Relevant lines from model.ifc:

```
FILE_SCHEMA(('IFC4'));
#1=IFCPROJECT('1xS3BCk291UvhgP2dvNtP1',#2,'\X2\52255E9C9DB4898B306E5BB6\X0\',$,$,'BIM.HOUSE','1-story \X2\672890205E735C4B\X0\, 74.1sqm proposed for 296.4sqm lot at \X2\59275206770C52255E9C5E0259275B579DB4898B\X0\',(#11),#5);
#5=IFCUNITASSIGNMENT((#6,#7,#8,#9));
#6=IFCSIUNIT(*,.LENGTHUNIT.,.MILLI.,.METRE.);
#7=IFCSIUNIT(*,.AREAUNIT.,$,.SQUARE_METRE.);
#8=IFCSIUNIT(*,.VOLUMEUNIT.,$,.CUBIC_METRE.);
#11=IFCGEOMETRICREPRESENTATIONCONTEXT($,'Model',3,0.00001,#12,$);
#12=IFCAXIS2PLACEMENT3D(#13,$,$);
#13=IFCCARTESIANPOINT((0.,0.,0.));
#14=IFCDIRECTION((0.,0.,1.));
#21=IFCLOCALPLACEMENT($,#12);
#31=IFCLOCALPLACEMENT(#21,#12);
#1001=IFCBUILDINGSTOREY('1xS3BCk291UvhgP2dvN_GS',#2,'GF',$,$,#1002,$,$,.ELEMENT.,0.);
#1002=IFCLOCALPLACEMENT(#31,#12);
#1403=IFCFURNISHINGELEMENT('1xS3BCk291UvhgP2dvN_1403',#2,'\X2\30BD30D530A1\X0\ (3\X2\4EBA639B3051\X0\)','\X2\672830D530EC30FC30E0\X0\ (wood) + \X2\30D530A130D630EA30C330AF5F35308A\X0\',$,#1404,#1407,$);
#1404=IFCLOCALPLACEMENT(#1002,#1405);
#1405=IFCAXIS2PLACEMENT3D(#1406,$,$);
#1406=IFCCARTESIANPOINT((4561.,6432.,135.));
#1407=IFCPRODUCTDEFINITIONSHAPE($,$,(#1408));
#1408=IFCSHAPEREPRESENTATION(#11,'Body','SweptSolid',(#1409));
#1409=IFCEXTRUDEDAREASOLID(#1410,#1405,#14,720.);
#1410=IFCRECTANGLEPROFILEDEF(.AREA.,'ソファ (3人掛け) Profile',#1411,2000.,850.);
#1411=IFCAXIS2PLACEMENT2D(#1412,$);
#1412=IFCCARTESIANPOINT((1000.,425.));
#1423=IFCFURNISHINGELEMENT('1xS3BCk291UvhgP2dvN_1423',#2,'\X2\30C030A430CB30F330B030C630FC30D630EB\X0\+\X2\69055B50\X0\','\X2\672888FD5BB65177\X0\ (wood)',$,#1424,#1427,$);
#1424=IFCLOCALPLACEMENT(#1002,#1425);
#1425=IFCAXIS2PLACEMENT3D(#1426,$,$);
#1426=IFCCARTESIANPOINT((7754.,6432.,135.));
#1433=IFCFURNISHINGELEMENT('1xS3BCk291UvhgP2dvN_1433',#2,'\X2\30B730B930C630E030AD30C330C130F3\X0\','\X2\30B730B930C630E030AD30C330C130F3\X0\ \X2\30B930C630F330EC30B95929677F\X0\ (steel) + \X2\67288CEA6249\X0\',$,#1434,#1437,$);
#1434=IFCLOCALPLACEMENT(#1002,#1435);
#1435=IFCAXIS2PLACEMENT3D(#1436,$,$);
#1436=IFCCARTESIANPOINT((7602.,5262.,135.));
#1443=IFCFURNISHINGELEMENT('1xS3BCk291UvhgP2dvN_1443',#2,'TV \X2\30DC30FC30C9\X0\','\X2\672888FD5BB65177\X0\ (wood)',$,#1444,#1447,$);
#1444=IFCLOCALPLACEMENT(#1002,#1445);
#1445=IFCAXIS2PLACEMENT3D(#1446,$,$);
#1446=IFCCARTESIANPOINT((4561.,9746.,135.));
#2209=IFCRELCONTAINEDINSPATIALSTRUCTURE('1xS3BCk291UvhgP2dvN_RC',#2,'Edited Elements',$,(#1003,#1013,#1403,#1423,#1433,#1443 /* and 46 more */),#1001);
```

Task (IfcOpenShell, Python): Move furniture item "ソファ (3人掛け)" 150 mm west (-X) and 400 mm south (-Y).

```python
import ifcopenshell
import ifcopenshell.api.geometry
import ifcopenshell.util.placement
import ifcopenshell.util.unit

model = ifcopenshell.open("model.ifc")
unit_scale = ifcopenshell.util.unit.calculate_unit_scale(model)

item = model.by_guid("1xS3BCk291UvhgP2dvN_1403")
matrix = ifcopenshell.util.placement.get_local_placement(item.ObjectPlacement)
matrix[0, 3] -= 0.15 / unit_scale
matrix[1, 3] -= 0.4 / unit_scale
ifcopenshell.api.geometry.edit_object_placement(model, product=item, matrix=matrix, is_si=False)

print(ifcopenshell.util.placement.get_local_placement(item.ObjectPlacement).round(3) + 0.0)

model.write("model_updated.ifc")
```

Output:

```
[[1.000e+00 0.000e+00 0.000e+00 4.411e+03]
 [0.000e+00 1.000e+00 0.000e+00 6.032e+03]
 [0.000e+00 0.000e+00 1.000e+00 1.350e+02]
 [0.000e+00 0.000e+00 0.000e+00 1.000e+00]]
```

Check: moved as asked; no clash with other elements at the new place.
